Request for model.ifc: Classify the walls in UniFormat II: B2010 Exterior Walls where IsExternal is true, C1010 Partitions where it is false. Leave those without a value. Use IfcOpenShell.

First a look at what the model holds.

```python
import ifcopenshell
import ifcopenshell.util.element

model = ifcopenshell.open("model.ifc")
print(model.schema)
print("classifications:", [c.Name for c in model.by_type("IfcClassification")])
values = [ifcopenshell.util.element.get_pset(e, "Pset_WallCommon", "IsExternal") for e in model.by_type("IfcWall")]
for value in (True, False, None):
    print("IsExternal", value, values.count(value))
```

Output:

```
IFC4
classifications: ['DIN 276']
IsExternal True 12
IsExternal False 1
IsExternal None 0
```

```python
import ifcopenshell
import ifcopenshell.api.classification
import ifcopenshell.util.element

model = ifcopenshell.open("model.ifc")

system = ifcopenshell.api.classification.add_classification(model, classification="UniFormat II")

walls = model.by_type("IfcWall")
external = {e: ifcopenshell.util.element.get_pset(e, "Pset_WallCommon", "IsExternal") for e in walls}
for flag, code, name in ((True, "B2010", "Exterior Walls"), (False, "C1010", "Partitions")):
    products = [e for e in walls if external[e] is flag]
    ifcopenshell.api.classification.add_reference(
        model, products=products, classification=system, identification=code, name=name
    )
    print(code, len(products))

model.write("model-out.ifc")
```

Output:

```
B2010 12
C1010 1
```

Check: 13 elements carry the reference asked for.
